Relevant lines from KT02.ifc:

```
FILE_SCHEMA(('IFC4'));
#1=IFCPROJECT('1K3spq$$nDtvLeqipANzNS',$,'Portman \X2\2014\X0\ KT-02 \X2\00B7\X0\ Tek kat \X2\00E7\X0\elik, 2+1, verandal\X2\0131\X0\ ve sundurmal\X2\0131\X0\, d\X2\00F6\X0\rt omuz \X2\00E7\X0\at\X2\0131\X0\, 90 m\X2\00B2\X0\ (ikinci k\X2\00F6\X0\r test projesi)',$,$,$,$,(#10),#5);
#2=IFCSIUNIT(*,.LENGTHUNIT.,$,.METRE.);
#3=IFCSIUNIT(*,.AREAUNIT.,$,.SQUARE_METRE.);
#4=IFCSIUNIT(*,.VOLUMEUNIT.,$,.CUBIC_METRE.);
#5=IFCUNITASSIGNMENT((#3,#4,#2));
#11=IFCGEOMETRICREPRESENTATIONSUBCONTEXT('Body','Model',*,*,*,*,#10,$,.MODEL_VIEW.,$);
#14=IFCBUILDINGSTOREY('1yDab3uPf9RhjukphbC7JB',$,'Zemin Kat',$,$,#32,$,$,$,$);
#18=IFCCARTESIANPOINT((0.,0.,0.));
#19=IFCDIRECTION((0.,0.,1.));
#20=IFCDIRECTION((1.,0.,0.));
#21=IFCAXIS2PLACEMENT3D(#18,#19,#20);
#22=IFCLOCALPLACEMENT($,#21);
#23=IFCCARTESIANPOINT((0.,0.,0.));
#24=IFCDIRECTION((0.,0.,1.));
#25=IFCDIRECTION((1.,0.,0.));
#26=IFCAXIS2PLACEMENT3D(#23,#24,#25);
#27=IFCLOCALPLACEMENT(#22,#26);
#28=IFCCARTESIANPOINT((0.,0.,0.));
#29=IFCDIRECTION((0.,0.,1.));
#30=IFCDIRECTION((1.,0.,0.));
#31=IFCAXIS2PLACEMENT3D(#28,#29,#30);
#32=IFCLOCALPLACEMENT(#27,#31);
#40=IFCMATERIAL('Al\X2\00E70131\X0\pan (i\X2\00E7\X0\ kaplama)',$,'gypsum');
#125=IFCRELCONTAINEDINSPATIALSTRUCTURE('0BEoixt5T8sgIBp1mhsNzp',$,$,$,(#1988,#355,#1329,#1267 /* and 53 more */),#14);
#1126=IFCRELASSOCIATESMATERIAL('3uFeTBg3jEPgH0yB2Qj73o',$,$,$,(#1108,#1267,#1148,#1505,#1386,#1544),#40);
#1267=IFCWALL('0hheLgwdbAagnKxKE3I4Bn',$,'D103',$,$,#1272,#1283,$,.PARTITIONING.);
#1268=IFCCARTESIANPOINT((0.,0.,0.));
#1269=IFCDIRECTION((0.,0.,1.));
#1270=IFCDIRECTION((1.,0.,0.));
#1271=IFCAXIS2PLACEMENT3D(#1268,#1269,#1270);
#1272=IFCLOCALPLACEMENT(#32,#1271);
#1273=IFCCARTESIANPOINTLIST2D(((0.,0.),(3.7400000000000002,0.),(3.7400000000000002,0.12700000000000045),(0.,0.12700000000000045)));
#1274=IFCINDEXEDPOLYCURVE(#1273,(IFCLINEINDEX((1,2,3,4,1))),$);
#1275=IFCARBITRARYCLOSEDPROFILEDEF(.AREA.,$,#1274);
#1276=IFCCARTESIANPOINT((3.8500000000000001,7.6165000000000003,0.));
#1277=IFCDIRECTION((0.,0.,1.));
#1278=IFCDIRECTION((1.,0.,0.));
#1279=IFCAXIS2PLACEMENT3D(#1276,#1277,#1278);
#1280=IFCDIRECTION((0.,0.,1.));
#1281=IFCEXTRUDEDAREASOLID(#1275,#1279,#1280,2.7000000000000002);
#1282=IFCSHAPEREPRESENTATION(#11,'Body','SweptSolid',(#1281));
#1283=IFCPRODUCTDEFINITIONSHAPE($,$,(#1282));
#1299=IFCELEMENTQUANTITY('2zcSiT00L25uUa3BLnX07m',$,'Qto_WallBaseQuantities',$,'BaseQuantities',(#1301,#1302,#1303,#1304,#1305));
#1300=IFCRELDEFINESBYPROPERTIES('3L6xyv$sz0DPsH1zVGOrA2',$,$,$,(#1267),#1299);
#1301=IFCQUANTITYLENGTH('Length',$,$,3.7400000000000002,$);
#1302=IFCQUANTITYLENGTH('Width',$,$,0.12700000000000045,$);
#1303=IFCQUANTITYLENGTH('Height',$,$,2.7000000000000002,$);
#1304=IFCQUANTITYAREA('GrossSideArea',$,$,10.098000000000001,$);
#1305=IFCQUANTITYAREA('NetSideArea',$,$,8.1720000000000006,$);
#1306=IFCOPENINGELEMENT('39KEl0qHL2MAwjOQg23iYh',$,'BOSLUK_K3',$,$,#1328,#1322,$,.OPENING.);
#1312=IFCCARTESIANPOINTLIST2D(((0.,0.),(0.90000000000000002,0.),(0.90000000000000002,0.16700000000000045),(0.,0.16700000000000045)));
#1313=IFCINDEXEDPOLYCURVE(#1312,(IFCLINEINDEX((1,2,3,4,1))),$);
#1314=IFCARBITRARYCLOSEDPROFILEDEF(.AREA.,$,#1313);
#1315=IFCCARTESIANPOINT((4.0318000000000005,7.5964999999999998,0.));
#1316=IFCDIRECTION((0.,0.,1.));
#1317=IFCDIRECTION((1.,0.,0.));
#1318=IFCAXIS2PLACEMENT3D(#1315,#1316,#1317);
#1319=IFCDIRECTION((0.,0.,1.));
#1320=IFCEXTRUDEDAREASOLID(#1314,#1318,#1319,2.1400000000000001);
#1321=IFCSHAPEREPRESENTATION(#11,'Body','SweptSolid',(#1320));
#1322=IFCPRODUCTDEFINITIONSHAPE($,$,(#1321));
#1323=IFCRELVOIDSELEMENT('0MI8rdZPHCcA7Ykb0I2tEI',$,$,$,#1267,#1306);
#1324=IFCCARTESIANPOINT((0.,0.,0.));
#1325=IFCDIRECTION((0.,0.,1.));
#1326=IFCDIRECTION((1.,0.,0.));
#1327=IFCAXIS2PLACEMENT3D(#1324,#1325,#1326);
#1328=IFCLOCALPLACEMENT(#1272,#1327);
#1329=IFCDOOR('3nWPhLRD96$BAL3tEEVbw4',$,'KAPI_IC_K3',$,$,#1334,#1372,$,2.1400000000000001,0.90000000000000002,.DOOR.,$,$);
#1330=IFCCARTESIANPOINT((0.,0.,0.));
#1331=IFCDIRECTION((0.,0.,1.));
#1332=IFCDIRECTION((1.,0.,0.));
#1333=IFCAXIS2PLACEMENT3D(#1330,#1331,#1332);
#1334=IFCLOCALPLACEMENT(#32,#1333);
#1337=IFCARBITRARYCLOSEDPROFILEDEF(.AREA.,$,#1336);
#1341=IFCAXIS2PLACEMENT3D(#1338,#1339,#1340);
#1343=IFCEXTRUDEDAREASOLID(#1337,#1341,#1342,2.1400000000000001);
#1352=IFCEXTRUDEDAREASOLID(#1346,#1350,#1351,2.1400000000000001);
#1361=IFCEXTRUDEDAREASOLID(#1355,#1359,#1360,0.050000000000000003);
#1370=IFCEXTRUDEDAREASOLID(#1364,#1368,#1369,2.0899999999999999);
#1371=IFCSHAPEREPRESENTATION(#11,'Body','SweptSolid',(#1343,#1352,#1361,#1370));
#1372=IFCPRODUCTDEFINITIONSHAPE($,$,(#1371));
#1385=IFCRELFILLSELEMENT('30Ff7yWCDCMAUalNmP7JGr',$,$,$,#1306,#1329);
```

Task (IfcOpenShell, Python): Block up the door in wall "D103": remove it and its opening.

```python
import ifcopenshell
import ifcopenshell.api.feature
import ifcopenshell.api.pset
import ifcopenshell.api.root
import ifcopenshell.geom
import ifcopenshell.util.element
import ifcopenshell.util.shape
import ifcopenshell.util.unit

model = ifcopenshell.open("KT02.ifc")
area_scale = ifcopenshell.util.unit.calculate_unit_scale(model, "AREAUNIT")
settings = ifcopenshell.geom.settings()


def volume(element):
    """Net volume in cubic metres, openings subtracted."""
    shape = ifcopenshell.geom.create_shape(settings, element)
    return ifcopenshell.util.shape.get_volume(shape.geometry)


door = model.by_guid("3nWPhLRD96$BAL3tEEVbw4")
opening = door.FillsVoids[0].RelatingOpeningElement
wall = opening.VoidsElements[0].RelatingBuildingElement
before = volume(wall)

ifcopenshell.api.root.remove_product(model, product=door)
ifcopenshell.api.feature.remove_feature(model, feature=opening)

after = volume(wall)
thickness = 0.127  # wall thickness in metres

# Update the wall's stored quantities.
qto = model.by_id(ifcopenshell.util.element.get_pset(wall, "Qto_WallBaseQuantities", should_inherit=False)["id"])
ifcopenshell.api.pset.edit_qto(model, qto=qto, properties={"NetSideArea": after / thickness / area_scale})

print(f"wall volume {before:.3f} -> {after:.3f} m3")

model.write("KT02_rev.ifc")
```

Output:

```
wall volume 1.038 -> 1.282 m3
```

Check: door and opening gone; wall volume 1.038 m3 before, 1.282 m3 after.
